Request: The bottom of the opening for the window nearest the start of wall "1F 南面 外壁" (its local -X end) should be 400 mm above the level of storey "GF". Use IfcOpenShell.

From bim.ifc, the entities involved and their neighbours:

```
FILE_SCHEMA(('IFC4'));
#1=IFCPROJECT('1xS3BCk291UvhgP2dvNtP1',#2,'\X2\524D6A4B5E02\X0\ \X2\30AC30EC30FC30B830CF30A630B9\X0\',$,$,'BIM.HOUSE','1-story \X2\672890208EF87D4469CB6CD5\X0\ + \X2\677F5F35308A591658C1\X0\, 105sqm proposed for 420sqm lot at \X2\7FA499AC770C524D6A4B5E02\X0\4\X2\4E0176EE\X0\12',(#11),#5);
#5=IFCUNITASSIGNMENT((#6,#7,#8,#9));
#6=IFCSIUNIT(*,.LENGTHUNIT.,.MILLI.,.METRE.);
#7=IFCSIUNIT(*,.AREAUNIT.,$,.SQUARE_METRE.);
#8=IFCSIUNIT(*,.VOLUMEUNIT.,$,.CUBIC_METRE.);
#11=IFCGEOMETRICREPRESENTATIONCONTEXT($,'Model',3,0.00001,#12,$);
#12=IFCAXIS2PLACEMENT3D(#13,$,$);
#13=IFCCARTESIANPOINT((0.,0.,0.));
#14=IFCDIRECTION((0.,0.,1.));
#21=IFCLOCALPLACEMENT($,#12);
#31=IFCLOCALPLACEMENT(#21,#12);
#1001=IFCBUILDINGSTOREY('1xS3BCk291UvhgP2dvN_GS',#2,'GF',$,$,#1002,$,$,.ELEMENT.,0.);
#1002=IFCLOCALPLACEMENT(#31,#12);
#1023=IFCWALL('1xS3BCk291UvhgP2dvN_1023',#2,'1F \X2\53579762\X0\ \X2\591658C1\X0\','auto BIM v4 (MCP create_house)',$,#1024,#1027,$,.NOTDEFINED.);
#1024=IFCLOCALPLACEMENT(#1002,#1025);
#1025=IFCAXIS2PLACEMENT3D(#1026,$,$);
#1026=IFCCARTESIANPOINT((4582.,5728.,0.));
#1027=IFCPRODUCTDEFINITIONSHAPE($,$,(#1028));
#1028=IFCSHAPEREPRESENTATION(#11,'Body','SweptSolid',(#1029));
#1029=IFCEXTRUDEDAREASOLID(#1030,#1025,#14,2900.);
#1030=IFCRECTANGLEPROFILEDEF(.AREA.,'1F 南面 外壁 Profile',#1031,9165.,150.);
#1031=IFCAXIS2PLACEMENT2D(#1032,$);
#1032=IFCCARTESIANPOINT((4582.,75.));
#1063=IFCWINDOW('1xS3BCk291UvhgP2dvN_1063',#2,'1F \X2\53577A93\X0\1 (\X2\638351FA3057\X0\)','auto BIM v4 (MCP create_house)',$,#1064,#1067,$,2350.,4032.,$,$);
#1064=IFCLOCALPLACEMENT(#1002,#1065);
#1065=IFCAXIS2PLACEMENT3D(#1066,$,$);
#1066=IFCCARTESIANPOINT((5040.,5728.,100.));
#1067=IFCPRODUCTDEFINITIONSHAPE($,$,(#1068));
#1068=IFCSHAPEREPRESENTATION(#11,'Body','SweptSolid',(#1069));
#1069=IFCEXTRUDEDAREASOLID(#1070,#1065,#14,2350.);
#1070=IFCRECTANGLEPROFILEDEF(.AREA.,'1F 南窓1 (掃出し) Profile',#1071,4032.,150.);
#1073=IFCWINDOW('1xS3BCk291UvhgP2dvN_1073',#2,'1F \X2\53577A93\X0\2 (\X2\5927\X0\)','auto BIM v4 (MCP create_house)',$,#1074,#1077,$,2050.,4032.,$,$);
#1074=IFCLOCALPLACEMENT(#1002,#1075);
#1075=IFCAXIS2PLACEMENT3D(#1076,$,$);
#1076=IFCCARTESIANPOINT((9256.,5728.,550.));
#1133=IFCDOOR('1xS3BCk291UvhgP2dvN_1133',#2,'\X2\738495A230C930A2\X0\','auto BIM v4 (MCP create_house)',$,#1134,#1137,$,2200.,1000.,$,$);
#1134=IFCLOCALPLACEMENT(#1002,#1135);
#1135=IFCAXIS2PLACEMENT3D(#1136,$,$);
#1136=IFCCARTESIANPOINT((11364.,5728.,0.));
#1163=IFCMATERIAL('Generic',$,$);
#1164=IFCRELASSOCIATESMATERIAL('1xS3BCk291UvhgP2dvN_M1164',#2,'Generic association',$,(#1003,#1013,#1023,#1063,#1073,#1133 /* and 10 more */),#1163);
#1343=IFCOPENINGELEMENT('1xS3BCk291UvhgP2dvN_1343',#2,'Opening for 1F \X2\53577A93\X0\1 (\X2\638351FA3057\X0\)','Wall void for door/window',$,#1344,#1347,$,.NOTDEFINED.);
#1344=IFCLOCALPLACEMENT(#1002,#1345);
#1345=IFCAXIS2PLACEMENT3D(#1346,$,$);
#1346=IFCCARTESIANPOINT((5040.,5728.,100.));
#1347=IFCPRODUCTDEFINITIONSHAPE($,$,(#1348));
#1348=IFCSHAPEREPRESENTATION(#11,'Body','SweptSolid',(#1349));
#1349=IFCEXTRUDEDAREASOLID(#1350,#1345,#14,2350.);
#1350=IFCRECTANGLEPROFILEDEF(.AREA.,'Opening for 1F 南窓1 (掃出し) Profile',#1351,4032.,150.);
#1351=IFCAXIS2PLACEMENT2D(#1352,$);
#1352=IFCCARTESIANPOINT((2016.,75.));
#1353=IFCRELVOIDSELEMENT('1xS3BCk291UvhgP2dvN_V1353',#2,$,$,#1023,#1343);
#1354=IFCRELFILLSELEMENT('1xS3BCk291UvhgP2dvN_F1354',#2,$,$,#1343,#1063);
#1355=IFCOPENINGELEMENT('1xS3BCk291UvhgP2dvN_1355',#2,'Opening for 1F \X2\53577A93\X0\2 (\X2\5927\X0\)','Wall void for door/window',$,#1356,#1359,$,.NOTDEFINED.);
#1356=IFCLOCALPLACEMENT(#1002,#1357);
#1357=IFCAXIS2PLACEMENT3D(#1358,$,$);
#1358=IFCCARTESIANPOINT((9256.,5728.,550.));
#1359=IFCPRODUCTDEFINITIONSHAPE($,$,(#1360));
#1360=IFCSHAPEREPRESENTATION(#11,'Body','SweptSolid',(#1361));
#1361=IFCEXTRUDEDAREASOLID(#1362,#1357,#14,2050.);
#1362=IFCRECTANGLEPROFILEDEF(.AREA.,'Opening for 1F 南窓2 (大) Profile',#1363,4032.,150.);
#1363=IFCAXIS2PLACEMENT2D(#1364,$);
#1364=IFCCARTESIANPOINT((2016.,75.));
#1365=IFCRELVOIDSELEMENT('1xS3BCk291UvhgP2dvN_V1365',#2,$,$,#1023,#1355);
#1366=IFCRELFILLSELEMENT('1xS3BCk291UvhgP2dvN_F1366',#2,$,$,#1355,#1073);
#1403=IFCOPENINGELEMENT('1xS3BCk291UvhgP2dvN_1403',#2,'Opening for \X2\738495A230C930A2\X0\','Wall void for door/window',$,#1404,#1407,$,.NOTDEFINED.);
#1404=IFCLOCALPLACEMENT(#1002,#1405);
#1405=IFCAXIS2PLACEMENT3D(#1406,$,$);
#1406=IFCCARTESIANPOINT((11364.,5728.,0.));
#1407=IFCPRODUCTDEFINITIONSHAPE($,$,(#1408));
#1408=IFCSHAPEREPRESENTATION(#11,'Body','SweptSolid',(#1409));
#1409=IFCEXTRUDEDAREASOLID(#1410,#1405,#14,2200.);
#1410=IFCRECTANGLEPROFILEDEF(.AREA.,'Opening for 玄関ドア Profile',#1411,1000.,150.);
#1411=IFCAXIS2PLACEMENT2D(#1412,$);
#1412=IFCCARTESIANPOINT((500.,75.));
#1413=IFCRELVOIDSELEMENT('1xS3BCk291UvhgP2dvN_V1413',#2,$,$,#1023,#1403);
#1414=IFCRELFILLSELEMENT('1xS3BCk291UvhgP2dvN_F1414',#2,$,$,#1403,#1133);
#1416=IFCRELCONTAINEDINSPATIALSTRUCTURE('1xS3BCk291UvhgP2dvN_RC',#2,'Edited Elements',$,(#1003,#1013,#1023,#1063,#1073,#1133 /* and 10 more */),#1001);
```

```python
import numpy as np
import ifcopenshell
import ifcopenshell.api.geometry
import ifcopenshell.geom
import ifcopenshell.util.element
import ifcopenshell.util.placement
import ifcopenshell.util.shape
import ifcopenshell.util.unit

model = ifcopenshell.open("bim.ifc")
unit_scale = ifcopenshell.util.unit.calculate_unit_scale(model)

window = model.by_guid("1xS3BCk291UvhgP2dvN_1063")
opening = window.FillsVoids[0].RelatingOpeningElement
storey = ifcopenshell.util.element.get_container(window, ifc_class="IfcBuildingStorey")
level = ifcopenshell.util.placement.get_local_placement(storey.ObjectPlacement)[2, 3]

# The opening's origin need not be at the sill, so measure its lowest point.
shape = ifcopenshell.geom.create_shape(ifcopenshell.geom.settings(), opening)
bottom = ifcopenshell.util.shape.get_shape_bottom_elevation(shape, shape.geometry) / unit_scale
dz = level + 400.0 - bottom

shift = np.array([0.0, 0.0, dz])
# The window is not placed relative to its opening, so move both.
for product in (opening, window):
    matrix = ifcopenshell.util.placement.get_local_placement(product.ObjectPlacement)
    matrix[:3, 3] += shift
    ifcopenshell.api.geometry.edit_object_placement(model, product=product, matrix=matrix, is_si=False)

print(f"moved by {dz * unit_scale:+.3f} m")

model.write("bim-out.ifc")
```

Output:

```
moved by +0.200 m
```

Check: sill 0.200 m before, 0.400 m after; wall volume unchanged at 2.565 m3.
